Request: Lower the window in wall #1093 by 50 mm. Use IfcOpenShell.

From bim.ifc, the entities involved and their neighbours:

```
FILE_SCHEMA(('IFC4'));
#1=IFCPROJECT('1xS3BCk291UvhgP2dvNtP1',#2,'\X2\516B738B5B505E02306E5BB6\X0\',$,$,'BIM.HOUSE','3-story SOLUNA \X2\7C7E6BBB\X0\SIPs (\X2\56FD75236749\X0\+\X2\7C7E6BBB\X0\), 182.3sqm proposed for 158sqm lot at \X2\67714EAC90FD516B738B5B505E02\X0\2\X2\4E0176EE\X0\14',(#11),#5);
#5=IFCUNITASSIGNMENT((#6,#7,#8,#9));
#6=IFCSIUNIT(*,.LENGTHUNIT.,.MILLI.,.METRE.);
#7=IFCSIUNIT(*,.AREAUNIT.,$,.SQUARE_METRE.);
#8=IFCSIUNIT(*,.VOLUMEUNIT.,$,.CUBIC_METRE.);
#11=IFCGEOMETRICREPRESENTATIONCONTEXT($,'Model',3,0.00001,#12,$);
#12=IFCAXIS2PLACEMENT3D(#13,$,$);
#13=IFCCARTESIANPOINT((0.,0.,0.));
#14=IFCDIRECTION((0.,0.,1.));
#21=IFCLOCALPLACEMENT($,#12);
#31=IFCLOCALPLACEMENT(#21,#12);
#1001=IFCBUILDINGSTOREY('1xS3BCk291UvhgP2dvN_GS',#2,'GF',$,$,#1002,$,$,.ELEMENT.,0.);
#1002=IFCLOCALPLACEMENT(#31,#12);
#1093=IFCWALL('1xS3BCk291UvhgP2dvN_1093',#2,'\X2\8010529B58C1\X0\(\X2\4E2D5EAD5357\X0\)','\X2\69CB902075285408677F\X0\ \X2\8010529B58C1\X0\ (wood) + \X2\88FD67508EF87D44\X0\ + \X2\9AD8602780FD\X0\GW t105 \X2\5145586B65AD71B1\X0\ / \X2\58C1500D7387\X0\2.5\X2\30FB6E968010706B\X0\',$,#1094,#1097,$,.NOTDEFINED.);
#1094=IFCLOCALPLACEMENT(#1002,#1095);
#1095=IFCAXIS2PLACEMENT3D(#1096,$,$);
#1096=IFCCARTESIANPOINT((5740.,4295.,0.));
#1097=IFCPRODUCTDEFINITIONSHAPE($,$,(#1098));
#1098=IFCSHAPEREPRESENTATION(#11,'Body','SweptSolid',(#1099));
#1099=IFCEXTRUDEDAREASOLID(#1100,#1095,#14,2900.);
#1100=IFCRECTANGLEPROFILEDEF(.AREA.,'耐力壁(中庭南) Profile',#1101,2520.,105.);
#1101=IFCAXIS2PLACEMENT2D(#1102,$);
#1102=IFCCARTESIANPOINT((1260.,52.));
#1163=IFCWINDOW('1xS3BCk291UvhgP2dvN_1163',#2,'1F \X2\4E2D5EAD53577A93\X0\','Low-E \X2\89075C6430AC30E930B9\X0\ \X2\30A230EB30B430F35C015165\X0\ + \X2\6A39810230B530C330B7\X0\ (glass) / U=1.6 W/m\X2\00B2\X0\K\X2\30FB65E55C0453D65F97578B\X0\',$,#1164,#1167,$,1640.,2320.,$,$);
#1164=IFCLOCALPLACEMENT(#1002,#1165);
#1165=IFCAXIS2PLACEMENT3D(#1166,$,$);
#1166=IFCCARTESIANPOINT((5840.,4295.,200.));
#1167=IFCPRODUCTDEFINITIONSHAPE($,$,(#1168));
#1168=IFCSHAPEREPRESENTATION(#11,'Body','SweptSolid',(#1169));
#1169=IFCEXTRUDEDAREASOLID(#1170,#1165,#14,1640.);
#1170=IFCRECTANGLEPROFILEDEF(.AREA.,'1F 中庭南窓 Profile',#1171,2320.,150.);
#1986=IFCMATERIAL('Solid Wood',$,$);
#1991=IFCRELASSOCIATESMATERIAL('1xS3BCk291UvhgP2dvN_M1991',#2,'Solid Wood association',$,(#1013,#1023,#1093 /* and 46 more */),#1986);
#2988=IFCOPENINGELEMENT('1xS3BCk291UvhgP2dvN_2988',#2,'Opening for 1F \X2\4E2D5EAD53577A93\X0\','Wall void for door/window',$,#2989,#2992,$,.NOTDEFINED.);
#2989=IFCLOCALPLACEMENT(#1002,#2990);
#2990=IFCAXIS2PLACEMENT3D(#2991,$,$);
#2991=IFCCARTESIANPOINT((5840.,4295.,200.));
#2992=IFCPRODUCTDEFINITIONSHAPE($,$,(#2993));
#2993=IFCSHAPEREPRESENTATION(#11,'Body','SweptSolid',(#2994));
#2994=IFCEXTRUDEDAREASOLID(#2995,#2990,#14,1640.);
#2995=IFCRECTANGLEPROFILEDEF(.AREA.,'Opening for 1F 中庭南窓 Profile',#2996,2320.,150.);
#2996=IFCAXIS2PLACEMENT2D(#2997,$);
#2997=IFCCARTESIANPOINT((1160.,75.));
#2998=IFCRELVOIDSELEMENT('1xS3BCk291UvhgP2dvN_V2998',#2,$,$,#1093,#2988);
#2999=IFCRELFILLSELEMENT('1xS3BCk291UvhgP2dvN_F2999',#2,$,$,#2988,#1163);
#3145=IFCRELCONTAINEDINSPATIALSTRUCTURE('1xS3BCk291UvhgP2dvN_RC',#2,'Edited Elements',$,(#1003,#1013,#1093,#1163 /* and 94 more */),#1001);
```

```python
import numpy as np
import ifcopenshell
import ifcopenshell.api.geometry
import ifcopenshell.util.placement
import ifcopenshell.util.unit

model = ifcopenshell.open("bim.ifc")
unit_scale = ifcopenshell.util.unit.calculate_unit_scale(model)

window = model.by_guid("1xS3BCk291UvhgP2dvN_1163")
opening = window.FillsVoids[0].RelatingOpeningElement
dz = -50.0

shift = np.array([0.0, 0.0, dz])
# The window is not placed relative to its opening, so move both.
for product in (opening, window):
    matrix = ifcopenshell.util.placement.get_local_placement(product.ObjectPlacement)
    matrix[:3, 3] += shift
    ifcopenshell.api.geometry.edit_object_placement(model, product=product, matrix=matrix, is_si=False)

print(f"moved by {dz * unit_scale:+.3f} m")

model.write("bim-out.ifc")
```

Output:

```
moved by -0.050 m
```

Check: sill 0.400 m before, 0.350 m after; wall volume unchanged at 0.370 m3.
